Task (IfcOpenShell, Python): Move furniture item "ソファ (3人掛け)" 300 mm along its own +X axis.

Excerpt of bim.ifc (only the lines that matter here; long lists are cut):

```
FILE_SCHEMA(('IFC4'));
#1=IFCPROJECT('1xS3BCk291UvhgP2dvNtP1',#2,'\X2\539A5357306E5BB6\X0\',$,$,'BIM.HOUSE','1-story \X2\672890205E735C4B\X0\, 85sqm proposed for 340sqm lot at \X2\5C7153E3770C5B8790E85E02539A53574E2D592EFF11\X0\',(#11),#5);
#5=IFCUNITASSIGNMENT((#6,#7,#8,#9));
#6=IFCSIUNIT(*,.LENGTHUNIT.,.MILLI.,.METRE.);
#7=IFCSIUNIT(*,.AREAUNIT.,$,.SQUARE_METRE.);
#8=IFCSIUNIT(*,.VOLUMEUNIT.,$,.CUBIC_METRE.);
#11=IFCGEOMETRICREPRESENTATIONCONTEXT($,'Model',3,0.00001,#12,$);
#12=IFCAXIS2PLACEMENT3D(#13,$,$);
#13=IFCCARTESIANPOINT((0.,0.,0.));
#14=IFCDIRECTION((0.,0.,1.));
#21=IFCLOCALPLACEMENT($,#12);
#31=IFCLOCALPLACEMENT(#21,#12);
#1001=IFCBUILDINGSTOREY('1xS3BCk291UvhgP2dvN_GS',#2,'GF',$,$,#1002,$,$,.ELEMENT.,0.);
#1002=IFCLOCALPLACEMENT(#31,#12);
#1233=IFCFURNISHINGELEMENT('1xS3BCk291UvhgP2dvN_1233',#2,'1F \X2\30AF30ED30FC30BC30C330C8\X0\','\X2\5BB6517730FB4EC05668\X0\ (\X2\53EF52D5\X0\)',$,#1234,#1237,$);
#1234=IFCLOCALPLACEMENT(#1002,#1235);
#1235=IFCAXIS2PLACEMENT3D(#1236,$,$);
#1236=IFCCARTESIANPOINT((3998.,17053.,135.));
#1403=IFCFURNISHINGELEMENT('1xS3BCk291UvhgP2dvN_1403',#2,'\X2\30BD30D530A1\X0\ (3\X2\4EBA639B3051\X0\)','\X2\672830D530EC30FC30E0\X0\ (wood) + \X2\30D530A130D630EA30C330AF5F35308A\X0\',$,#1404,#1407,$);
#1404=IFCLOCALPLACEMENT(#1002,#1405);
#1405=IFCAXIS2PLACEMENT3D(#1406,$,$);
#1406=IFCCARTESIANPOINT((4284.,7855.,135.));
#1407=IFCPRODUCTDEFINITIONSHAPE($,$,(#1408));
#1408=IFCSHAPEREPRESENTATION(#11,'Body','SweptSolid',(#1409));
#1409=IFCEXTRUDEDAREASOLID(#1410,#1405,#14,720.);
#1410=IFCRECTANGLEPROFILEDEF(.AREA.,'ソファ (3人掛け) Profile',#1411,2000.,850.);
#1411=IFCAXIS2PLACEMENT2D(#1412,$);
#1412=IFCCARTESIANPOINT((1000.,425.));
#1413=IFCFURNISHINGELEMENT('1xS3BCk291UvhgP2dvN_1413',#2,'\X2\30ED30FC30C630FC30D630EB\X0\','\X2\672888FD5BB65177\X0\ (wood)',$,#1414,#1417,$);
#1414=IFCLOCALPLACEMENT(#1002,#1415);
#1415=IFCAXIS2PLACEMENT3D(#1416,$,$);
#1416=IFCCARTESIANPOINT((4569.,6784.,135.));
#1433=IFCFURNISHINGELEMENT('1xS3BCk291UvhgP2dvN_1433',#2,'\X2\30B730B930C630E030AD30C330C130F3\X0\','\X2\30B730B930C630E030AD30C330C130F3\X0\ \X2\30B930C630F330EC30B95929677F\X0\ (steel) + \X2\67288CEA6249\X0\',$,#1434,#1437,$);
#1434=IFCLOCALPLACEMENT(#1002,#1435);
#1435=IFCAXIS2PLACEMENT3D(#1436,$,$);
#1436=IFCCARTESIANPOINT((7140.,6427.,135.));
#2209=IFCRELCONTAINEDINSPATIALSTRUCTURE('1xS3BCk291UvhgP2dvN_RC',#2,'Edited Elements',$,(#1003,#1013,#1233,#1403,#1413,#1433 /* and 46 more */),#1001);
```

```python
import ifcopenshell
import ifcopenshell.api.geometry
import ifcopenshell.util.placement

model = ifcopenshell.open("bim.ifc")

item = model.by_guid("1xS3BCk291UvhgP2dvN_1403")
matrix = ifcopenshell.util.placement.get_local_placement(item.ObjectPlacement)
matrix[:3, 3] += matrix[:3, 0] * 300.0
ifcopenshell.api.geometry.edit_object_placement(model, product=item, matrix=matrix, is_si=False)

print(ifcopenshell.util.placement.get_local_placement(item.ObjectPlacement).round(3) + 0.0)

model.write("bim_v2.ifc")
```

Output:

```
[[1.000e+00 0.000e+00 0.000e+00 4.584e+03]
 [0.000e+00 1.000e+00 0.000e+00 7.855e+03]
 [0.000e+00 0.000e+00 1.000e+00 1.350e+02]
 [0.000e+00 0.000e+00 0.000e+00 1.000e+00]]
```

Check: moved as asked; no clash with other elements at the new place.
